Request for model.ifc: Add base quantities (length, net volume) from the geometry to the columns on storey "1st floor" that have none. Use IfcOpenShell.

First a look at what the model holds.

```python
import ifcopenshell
import ifcopenshell.util.element
import ifcopenshell.util.unit

model = ifcopenshell.open("model.ifc")
print(model.schema)
for unit_type in ("LENGTHUNIT", "AREAUNIT", "VOLUMEUNIT"):
    print(unit_type, ifcopenshell.util.unit.calculate_unit_scale(model, unit_type))
storey = next(s for s in model.by_type("IfcBuildingStorey") if s.Name == "1st floor")
columns = [e for e in ifcopenshell.util.element.get_decomposition(storey) if e.is_a("IfcColumn")]
for e in sorted(columns, key=lambda e: e.id()):
    print(e.id(), e.is_a(), e.Name, list(ifcopenshell.util.element.get_psets(e, qtos_only=True)), sep=" | ")
```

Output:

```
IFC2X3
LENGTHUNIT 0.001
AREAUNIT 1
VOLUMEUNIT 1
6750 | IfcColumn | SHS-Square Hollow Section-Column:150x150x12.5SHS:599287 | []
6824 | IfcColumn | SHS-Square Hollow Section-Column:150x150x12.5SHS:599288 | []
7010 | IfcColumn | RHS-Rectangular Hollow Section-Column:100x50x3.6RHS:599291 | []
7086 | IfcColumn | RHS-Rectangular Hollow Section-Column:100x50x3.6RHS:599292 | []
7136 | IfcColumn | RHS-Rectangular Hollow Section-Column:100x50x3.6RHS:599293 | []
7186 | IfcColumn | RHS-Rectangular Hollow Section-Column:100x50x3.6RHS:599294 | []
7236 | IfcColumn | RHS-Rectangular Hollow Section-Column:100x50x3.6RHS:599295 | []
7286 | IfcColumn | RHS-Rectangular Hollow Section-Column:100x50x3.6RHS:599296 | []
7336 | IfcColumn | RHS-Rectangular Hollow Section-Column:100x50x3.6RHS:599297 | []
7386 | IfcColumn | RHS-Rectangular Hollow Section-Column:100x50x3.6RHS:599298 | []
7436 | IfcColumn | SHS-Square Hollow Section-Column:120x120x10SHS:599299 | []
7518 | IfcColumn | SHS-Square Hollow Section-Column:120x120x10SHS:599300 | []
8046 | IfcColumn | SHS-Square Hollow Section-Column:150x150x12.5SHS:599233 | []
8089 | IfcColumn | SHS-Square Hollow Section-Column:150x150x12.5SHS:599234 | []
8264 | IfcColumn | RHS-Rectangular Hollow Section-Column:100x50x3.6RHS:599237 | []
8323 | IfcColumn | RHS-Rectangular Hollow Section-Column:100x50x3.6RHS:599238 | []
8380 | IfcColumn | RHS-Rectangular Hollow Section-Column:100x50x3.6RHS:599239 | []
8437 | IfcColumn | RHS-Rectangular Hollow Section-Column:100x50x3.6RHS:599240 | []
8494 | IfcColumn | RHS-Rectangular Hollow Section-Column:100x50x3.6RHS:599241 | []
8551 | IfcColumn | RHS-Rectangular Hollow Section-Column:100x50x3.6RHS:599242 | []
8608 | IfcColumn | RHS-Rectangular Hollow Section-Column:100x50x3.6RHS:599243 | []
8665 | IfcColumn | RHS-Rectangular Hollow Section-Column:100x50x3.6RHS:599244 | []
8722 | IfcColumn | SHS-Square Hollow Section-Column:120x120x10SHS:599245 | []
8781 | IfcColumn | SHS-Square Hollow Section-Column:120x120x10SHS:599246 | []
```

```python
import ifcopenshell
import ifcopenshell.api.pset
import ifcopenshell.geom
import ifcopenshell.util.element
import ifcopenshell.util.shape
import ifcopenshell.util.unit

model = ifcopenshell.open("model.ifc")
unit_scale = ifcopenshell.util.unit.calculate_unit_scale(model)
volume_scale = ifcopenshell.util.unit.calculate_unit_scale(model, "VOLUMEUNIT")
settings = ifcopenshell.geom.settings()

storey = next(s for s in model.by_type("IfcBuildingStorey") if s.Name == "1st floor")
columns = [e for e in ifcopenshell.util.element.get_decomposition(storey) if e.is_a("IfcColumn")]

for e in sorted(columns, key=lambda e: e.id()):
    if ifcopenshell.util.element.get_psets(e, qtos_only=True, should_inherit=False):
        continue
    # Geometry comes back in metres, in the element's own axes.
    shape = ifcopenshell.geom.create_shape(settings, e)
    values = {
        "Length": ifcopenshell.util.shape.get_z(shape.geometry) / unit_scale,
        "NetVolume": ifcopenshell.util.shape.get_volume(shape.geometry) / volume_scale,
    }
    qto = ifcopenshell.api.pset.add_qto(model, product=e, name="BaseQuantities")
    ifcopenshell.api.pset.edit_qto(model, qto=qto, properties=values)
    print(e.id(), {k: round(v, 3) for k, v in values.items()})

model.write("model_edited.ifc")
```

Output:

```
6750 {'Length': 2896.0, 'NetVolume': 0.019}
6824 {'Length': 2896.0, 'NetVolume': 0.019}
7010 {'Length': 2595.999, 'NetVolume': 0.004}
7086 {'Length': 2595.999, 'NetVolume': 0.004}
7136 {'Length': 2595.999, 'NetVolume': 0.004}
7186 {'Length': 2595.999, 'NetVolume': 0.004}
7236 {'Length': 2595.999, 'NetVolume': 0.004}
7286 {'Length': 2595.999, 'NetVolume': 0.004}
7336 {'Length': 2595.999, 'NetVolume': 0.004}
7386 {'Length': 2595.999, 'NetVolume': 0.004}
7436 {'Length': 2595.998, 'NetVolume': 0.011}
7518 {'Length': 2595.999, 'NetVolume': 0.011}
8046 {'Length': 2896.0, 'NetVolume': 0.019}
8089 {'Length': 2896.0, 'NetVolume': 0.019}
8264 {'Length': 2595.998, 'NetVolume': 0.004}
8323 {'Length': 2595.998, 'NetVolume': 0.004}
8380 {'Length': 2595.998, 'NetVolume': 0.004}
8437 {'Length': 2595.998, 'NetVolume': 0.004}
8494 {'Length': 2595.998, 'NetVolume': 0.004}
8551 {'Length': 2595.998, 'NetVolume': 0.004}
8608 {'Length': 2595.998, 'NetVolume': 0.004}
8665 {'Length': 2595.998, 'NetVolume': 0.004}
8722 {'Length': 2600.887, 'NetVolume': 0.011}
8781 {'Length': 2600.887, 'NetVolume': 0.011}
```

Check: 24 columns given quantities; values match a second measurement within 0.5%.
